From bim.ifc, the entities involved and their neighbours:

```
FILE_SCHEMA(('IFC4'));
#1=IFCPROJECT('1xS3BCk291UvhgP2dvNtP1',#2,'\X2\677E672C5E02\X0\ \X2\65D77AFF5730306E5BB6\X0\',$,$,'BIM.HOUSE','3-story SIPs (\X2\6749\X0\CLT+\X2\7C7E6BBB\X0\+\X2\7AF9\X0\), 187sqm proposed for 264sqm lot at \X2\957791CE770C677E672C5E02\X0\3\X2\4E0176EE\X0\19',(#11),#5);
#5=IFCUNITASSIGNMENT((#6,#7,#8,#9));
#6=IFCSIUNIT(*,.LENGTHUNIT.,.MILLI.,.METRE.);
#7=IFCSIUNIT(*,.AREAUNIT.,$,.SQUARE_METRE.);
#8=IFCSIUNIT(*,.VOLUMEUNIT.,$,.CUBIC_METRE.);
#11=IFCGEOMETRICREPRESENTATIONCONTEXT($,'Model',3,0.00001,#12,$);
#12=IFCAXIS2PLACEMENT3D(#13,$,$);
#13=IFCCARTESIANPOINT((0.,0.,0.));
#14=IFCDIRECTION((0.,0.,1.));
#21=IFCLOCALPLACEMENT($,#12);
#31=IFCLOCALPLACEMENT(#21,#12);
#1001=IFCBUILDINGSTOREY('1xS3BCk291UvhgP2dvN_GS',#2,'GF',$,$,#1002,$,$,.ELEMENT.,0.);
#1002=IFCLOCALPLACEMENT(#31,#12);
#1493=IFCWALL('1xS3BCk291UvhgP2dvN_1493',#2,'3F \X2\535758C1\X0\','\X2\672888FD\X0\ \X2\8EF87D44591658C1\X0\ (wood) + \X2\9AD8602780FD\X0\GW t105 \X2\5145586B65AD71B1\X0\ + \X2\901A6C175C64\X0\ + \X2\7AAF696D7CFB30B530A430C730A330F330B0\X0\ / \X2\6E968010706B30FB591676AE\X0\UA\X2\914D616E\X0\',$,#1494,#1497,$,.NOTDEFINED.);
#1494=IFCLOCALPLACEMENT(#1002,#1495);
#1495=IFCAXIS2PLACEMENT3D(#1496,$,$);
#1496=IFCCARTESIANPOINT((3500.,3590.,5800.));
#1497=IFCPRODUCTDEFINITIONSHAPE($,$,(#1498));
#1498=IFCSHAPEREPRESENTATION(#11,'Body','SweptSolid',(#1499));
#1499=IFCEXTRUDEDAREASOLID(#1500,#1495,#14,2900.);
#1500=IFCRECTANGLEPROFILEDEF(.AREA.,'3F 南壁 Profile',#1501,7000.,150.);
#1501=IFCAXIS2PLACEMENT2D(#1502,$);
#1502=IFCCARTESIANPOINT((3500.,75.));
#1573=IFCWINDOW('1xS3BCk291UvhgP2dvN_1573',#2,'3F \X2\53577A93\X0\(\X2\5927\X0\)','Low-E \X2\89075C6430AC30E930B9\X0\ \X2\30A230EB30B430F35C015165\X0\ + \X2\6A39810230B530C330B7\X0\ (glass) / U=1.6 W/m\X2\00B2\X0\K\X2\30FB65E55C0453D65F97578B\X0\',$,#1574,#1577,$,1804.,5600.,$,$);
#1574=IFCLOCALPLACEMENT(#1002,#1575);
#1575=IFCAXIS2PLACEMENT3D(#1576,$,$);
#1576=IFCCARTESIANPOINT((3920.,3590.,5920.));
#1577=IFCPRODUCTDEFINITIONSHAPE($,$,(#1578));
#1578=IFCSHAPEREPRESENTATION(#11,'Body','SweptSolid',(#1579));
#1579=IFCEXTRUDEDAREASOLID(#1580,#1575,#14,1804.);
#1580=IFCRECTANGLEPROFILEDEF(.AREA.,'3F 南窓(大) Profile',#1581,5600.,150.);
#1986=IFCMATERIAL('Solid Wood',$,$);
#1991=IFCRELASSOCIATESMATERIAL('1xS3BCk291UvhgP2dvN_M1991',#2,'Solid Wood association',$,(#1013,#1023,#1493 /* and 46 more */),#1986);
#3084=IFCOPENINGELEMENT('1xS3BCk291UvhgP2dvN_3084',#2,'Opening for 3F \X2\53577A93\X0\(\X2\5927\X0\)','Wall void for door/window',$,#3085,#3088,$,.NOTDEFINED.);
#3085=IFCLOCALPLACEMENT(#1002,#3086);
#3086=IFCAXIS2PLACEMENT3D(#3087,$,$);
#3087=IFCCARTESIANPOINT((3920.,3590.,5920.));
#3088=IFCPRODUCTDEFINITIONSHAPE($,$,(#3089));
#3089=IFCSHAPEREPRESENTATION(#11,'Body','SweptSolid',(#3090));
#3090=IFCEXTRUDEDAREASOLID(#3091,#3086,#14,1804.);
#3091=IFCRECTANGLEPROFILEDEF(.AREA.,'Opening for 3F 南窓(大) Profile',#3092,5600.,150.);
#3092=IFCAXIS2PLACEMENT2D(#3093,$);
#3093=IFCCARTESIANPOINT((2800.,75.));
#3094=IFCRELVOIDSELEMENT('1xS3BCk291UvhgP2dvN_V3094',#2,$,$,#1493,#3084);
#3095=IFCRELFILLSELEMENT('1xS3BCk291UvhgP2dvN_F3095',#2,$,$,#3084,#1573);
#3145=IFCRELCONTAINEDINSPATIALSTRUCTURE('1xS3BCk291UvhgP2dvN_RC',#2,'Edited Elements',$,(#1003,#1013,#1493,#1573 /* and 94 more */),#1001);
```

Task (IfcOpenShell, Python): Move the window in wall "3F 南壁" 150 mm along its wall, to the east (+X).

```python
import ifcopenshell
import ifcopenshell.api.geometry
import ifcopenshell.util.placement

model = ifcopenshell.open("bim.ifc")

window = model.by_guid("1xS3BCk291UvhgP2dvN_1573")
opening = window.FillsVoids[0].RelatingOpeningElement
wall = opening.VoidsElements[0].RelatingBuildingElement

wall_matrix = ifcopenshell.util.placement.get_local_placement(wall.ObjectPlacement)
shift = wall_matrix[:3, 0] * 150.0
before = ifcopenshell.util.placement.get_local_placement(window.ObjectPlacement)[:3, 3].copy()

# The window is not placed relative to its opening, so move both.
for product in (opening, window):
    matrix = ifcopenshell.util.placement.get_local_placement(product.ObjectPlacement)
    matrix[:3, 3] += shift
    ifcopenshell.api.geometry.edit_object_placement(model, product=product, matrix=matrix, is_si=False)

after = ifcopenshell.util.placement.get_local_placement(window.ObjectPlacement)[:3, 3]
print("window moved by", (after - before).round(3) + 0.0)

model.write("bim_edited.ifc")
```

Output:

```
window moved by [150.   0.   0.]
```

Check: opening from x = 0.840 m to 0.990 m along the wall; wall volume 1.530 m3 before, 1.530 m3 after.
